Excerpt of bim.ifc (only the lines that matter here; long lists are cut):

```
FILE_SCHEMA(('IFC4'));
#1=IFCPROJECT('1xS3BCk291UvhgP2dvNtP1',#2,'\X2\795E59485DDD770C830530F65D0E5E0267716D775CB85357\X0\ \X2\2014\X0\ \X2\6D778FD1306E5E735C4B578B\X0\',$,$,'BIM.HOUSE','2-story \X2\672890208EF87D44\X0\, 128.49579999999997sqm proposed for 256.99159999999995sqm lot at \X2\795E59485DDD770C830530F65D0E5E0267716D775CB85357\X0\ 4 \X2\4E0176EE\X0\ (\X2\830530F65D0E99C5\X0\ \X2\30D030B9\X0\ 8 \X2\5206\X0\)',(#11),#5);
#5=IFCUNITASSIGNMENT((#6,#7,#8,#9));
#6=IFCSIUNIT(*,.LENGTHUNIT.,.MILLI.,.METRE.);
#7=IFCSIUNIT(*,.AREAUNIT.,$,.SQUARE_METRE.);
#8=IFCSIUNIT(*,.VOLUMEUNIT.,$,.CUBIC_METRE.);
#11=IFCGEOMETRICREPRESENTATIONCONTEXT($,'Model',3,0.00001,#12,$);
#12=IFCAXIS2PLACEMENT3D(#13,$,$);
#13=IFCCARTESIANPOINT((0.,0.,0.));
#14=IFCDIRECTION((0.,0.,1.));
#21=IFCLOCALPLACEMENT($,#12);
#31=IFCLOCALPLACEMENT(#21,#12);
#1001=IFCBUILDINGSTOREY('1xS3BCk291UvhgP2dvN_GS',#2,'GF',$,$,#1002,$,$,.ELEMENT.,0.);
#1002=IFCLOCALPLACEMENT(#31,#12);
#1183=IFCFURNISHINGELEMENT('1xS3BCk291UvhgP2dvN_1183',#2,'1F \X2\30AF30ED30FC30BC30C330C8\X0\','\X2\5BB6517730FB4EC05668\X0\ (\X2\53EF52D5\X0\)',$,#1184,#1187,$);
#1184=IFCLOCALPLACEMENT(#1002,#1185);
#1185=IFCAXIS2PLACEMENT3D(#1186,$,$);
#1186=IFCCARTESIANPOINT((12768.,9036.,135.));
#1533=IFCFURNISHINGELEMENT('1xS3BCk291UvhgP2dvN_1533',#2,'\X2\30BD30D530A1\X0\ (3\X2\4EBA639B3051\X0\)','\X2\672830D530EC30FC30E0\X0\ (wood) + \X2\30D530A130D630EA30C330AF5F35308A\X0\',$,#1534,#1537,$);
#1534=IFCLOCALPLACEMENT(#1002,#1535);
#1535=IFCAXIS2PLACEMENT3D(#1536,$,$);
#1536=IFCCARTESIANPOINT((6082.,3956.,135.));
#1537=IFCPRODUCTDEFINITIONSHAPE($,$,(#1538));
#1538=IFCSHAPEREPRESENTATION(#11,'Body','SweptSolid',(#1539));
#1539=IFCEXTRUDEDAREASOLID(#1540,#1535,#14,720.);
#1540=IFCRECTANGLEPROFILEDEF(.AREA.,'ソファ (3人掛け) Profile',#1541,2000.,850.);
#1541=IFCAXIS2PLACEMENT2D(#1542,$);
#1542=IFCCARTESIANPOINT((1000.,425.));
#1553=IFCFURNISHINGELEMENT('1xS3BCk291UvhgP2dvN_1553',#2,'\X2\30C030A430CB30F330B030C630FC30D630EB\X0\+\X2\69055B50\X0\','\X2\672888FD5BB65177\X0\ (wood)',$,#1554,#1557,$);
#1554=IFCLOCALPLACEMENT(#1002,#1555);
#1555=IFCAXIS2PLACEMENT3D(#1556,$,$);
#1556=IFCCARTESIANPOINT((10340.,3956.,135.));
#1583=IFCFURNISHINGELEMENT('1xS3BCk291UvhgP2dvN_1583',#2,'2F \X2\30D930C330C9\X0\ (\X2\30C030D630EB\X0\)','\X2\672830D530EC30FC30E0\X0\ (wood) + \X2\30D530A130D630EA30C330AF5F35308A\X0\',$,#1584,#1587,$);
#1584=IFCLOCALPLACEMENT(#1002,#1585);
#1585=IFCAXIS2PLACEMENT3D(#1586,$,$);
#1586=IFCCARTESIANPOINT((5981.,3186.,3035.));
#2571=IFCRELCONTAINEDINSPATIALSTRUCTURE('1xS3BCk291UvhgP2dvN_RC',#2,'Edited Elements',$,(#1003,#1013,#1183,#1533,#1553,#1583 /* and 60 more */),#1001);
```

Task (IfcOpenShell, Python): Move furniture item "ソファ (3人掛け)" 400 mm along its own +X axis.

```python
import ifcopenshell
import ifcopenshell.api.geometry
import ifcopenshell.util.placement
import ifcopenshell.util.unit

model = ifcopenshell.open("bim.ifc")
unit_scale = ifcopenshell.util.unit.calculate_unit_scale(model)

item = model.by_guid("1xS3BCk291UvhgP2dvN_1533")
matrix = ifcopenshell.util.placement.get_local_placement(item.ObjectPlacement)
matrix[:3, 3] += matrix[:3, 0] * 0.4 / unit_scale
ifcopenshell.api.geometry.edit_object_placement(model, product=item, matrix=matrix, is_si=False)

print(ifcopenshell.util.placement.get_local_placement(item.ObjectPlacement).round(3) + 0.0)

model.write("bim_updated.ifc")
```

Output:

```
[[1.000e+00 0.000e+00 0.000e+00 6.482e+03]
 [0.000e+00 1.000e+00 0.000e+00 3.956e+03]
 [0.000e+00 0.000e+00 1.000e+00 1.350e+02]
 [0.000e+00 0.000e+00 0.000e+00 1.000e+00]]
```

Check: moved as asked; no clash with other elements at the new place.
